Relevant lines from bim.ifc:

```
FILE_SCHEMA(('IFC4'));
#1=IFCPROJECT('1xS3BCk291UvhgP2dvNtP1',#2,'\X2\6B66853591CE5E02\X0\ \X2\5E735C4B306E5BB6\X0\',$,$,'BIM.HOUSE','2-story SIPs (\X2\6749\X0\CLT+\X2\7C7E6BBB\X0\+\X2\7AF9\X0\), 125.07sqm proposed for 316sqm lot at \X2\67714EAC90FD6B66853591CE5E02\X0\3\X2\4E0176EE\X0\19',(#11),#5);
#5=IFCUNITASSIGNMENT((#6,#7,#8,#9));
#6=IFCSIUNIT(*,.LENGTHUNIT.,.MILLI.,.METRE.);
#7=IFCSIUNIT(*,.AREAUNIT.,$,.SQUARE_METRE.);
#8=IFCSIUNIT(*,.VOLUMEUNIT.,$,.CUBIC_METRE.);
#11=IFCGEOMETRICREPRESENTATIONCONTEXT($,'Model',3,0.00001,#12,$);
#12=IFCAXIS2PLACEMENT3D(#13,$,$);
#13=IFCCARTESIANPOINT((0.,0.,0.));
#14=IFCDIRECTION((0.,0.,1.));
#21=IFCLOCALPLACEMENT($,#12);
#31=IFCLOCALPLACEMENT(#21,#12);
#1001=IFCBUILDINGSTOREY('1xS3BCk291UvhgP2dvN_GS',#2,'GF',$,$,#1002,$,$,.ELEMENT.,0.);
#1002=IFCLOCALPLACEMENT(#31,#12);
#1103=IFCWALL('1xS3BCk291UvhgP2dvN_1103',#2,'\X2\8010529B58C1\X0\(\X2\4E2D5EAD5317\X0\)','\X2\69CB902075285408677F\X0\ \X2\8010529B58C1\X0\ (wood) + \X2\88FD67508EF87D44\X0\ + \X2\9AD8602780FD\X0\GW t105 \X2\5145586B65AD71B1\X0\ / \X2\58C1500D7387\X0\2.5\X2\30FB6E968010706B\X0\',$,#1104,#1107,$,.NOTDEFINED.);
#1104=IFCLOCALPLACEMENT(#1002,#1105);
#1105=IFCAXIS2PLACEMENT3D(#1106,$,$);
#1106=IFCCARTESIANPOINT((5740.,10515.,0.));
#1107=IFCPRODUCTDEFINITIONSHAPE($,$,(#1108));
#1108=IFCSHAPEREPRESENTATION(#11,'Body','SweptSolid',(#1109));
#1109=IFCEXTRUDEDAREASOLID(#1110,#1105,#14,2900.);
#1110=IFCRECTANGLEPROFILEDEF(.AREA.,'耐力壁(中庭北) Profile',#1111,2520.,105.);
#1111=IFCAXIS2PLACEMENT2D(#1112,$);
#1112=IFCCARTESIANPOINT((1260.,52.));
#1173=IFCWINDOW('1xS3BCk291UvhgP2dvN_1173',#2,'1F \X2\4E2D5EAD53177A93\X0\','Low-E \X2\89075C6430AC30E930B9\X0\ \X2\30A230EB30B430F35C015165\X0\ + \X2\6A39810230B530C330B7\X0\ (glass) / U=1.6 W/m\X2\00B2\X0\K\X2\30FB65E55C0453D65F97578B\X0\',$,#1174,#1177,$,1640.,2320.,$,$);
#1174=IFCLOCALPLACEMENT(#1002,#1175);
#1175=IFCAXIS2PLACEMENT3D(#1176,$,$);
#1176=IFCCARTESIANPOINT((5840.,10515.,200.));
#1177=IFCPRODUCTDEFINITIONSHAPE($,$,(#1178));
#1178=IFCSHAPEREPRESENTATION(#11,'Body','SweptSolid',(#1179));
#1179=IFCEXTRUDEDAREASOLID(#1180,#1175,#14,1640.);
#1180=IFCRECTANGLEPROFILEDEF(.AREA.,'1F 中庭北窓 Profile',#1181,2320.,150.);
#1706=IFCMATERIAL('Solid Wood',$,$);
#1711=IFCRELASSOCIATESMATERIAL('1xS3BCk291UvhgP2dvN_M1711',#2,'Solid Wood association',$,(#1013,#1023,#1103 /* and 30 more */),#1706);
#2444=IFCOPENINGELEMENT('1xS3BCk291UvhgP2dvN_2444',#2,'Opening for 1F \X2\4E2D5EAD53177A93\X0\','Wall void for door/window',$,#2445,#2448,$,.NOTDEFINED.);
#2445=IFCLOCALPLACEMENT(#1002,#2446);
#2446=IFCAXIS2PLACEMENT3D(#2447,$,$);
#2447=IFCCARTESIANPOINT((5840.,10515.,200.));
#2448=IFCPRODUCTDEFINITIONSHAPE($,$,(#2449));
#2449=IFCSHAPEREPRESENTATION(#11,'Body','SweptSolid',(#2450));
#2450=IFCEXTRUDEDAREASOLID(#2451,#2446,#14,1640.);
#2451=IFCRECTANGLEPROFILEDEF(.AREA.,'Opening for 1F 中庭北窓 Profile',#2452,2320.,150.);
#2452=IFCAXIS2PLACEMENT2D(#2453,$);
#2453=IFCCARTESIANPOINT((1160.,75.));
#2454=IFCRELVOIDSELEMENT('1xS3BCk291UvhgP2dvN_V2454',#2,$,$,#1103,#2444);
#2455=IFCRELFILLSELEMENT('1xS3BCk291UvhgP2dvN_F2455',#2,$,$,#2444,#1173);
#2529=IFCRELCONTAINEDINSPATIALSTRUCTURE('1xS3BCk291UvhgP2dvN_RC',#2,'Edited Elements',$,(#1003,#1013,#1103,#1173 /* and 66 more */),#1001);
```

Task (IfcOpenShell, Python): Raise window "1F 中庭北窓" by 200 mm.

```python
import numpy as np
import ifcopenshell
import ifcopenshell.api.geometry
import ifcopenshell.util.placement
import ifcopenshell.util.unit

model = ifcopenshell.open("bim.ifc")
unit_scale = ifcopenshell.util.unit.calculate_unit_scale(model)

window = model.by_guid("1xS3BCk291UvhgP2dvN_1173")
opening = window.FillsVoids[0].RelatingOpeningElement
dz = 0.2 / unit_scale

shift = np.array([0.0, 0.0, dz])
# The window is not placed relative to its opening, so move both.
for product in (opening, window):
    matrix = ifcopenshell.util.placement.get_local_placement(product.ObjectPlacement)
    matrix[:3, 3] += shift
    ifcopenshell.api.geometry.edit_object_placement(model, product=product, matrix=matrix, is_si=False)

print(f"moved by {dz * unit_scale:+.3f} m")

model.write("bim_rev.ifc")
```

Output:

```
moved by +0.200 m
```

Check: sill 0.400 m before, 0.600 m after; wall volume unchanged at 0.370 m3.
